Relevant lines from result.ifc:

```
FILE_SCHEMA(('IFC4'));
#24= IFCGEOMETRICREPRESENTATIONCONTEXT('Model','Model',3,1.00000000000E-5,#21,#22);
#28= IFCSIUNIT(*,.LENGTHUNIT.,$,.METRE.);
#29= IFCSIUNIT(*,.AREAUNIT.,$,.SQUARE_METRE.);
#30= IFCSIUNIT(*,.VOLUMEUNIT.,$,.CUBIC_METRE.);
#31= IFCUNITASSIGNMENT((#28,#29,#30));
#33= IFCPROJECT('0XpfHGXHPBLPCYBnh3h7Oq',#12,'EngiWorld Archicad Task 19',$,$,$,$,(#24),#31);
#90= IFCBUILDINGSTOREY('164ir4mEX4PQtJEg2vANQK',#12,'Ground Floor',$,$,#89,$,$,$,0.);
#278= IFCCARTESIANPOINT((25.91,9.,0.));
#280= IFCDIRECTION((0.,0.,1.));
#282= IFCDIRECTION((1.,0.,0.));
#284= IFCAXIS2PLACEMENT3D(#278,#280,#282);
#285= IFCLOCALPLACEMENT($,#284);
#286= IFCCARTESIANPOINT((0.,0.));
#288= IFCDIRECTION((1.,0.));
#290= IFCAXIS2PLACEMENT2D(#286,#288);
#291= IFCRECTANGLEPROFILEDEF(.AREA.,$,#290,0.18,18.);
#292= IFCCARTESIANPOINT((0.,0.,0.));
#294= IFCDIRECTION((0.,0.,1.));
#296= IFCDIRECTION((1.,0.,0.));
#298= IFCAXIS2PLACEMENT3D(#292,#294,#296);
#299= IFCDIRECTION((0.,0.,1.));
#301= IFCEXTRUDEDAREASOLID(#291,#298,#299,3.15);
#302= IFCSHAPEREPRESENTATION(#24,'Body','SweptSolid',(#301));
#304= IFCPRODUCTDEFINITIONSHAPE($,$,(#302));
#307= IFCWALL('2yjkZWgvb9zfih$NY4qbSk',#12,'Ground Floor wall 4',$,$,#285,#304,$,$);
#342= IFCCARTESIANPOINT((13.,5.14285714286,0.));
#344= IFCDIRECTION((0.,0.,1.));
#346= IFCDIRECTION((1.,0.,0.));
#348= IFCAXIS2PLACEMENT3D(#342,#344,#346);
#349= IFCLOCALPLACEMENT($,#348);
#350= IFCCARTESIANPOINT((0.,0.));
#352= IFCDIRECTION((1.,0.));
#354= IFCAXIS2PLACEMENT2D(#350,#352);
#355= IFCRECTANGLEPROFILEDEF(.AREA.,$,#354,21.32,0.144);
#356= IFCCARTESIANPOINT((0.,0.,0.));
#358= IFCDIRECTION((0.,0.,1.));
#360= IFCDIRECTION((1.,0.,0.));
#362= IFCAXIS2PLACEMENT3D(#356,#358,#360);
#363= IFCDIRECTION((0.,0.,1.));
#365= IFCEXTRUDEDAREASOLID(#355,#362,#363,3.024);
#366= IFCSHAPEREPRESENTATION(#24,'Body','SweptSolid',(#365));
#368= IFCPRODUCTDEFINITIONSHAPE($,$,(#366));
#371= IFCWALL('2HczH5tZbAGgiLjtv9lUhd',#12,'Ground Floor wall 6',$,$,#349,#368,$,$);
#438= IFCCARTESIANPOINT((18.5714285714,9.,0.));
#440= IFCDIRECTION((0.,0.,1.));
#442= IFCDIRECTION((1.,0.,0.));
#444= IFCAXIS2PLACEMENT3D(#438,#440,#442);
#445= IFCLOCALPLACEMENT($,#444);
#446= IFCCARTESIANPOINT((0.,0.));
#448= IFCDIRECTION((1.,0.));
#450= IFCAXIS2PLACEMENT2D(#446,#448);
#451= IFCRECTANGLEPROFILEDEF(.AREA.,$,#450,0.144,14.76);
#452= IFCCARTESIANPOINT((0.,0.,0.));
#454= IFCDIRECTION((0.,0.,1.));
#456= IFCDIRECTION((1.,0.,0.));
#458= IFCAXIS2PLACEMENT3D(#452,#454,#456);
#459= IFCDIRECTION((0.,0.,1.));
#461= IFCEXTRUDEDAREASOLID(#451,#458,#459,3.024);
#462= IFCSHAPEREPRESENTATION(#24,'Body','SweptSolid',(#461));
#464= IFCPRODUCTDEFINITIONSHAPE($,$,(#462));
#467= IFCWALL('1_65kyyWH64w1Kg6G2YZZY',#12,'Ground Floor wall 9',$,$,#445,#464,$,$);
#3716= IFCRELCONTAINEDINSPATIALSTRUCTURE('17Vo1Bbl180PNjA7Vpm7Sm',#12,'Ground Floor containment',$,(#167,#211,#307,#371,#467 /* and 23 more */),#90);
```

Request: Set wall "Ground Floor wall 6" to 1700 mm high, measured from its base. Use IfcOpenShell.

```python
import ifcopenshell
import ifcopenshell.geom
import ifcopenshell.util.shape
import ifcopenshell.util.unit

model = ifcopenshell.open("result.ifc")
unit_scale = ifcopenshell.util.unit.calculate_unit_scale(model)
settings = ifcopenshell.geom.settings()


def volume(element):
    """Net volume in cubic metres, openings subtracted."""
    shape = ifcopenshell.geom.create_shape(settings, element)
    return ifcopenshell.util.shape.get_volume(shape.geometry)


wall = model.by_guid("2HczH5tZbAGgiLjtv9lUhd")
before = volume(wall)

body = next(r for r in wall.Representation.Representations if r.RepresentationIdentifier == "Body")
solid = body.Items[0]
old_height = solid.Depth
solid.Depth = 1.7 / unit_scale
after = volume(wall)

print(f"height {old_height:g} -> {solid.Depth:g}, volume {before:.3f} -> {after:.3f} m3")

model.write("result_updated.ifc")
```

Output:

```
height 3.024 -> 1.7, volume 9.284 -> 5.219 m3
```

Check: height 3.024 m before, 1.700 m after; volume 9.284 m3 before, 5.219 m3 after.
